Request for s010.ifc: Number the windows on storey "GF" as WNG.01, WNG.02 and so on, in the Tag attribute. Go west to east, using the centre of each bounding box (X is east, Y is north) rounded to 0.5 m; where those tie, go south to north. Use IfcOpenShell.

First a look at what the model holds.

```python
import ifcopenshell
import ifcopenshell.util.element
import ifcopenshell.util.placement

model = ifcopenshell.open("s010.ifc")
print(model.schema)
storey = next(s for s in model.by_type("IfcBuildingStorey") if s.Name == "GF")
windows = [e for e in ifcopenshell.util.element.get_decomposition(storey) if e.is_a("IfcWindow")]
for e in sorted(windows, key=lambda e: e.id()):
    origin = ifcopenshell.util.placement.get_local_placement(e.ObjectPlacement)[:3, 3]
    print(e.id(), e.Tag, e.Name, origin.round(2) + 0.0, sep=" | ")
```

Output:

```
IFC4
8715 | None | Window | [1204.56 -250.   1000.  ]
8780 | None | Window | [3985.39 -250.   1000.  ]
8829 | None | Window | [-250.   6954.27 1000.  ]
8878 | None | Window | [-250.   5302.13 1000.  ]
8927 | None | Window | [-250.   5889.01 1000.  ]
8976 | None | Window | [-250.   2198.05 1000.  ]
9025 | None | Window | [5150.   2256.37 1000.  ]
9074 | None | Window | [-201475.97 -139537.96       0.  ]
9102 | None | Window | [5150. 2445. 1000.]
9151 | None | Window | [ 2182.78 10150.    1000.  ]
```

```python
import ifcopenshell
import ifcopenshell.geom
import ifcopenshell.util.element
import ifcopenshell.util.shape

model = ifcopenshell.open("s010.ifc")
settings = ifcopenshell.geom.settings()
settings.set("use-world-coords", True)


def centre(element):
    shape = ifcopenshell.geom.create_shape(settings, element)
    return ifcopenshell.util.shape.get_bbox_centroid(shape.geometry)


storey = next(s for s in model.by_type("IfcBuildingStorey") if s.Name == "GF")
windows = [e for e in ifcopenshell.util.element.get_decomposition(storey) if e.is_a("IfcWindow")]

# Insertion points can sit at a corner or the storey origin, so sort by the geometry (in metres).
centres = {e: centre(e) for e in windows}
windows.sort(key=lambda e: (round(centres[e][0] / 0.5), centres[e][1]))

for i, e in enumerate(windows, start=1):
    number = f"WNG.{i:02d}"
    e.Tag = number
    print(e.id(), number)

model.write("s010_rev.ifc")
```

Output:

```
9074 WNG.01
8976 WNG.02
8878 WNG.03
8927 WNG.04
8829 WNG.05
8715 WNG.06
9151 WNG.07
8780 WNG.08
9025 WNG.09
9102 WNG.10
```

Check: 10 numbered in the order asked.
